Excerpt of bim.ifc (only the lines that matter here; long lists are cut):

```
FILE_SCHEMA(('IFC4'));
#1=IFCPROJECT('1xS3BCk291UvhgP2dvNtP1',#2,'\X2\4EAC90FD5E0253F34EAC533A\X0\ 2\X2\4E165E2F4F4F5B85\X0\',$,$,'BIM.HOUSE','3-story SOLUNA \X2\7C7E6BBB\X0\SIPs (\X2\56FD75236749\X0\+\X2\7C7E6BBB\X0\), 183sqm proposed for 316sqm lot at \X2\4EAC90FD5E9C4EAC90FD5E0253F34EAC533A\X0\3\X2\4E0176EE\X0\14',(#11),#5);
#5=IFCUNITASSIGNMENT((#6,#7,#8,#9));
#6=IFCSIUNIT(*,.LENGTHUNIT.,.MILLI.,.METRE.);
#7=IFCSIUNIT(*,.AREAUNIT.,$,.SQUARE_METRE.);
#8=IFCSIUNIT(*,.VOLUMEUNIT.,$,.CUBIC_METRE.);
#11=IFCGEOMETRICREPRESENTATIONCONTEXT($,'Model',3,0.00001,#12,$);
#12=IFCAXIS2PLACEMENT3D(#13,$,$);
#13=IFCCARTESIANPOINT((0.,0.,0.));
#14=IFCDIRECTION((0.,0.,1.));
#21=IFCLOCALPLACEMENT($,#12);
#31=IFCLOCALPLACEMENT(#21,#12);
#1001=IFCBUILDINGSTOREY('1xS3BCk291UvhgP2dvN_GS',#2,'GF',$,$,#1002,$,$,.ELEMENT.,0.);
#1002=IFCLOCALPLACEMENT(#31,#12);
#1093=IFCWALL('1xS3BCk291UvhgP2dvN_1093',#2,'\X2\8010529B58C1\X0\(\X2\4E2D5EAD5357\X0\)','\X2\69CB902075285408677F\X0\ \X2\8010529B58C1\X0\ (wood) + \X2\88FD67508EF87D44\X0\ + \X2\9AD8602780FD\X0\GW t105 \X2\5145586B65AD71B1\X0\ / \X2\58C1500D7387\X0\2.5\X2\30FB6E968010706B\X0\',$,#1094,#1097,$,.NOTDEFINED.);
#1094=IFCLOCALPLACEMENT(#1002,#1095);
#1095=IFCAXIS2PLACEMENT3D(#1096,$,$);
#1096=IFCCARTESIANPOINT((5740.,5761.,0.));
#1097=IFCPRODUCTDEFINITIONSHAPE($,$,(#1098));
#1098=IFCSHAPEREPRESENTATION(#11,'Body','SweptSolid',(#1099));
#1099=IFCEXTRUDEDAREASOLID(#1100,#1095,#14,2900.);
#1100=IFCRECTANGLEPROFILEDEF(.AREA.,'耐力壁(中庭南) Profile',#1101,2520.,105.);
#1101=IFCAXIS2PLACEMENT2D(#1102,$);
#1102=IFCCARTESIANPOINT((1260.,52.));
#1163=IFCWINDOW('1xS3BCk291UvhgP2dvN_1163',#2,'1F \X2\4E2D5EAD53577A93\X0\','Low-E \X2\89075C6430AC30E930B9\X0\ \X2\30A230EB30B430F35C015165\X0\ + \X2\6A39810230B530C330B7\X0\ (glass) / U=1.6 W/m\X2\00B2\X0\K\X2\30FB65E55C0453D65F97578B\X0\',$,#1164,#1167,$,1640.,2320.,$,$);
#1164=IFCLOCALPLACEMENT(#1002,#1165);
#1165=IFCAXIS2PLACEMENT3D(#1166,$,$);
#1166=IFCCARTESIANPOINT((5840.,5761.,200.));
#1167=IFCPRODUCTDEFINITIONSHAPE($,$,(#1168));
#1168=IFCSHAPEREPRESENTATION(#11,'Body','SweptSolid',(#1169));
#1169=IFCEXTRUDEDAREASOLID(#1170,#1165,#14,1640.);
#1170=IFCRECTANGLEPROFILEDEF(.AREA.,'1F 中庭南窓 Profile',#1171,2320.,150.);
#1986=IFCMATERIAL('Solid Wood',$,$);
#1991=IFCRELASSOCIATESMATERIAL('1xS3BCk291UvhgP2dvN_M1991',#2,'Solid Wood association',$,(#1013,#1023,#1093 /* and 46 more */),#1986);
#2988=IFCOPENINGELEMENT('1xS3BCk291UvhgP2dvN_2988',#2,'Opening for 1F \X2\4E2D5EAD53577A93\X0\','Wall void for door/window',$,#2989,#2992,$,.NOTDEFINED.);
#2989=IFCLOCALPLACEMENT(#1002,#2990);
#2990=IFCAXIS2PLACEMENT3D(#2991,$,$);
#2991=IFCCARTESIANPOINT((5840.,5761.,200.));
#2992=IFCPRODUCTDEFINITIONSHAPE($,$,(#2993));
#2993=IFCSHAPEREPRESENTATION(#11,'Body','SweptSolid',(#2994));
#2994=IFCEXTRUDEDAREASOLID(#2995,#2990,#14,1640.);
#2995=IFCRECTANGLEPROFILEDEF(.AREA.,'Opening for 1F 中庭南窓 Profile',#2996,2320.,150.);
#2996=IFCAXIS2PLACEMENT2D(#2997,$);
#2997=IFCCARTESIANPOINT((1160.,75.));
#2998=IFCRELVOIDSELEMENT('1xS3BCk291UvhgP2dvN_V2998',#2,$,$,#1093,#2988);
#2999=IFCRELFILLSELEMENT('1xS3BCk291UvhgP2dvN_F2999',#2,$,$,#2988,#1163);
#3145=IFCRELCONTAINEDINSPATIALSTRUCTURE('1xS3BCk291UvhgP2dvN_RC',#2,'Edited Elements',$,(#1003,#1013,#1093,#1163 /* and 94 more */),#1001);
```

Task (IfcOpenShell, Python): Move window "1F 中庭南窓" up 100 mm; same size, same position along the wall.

```python
import numpy as np
import ifcopenshell
import ifcopenshell.api.geometry
import ifcopenshell.util.placement
import ifcopenshell.util.unit

model = ifcopenshell.open("bim.ifc")
unit_scale = ifcopenshell.util.unit.calculate_unit_scale(model)

window = model.by_guid("1xS3BCk291UvhgP2dvN_1163")
opening = window.FillsVoids[0].RelatingOpeningElement
dz = 0.1 / unit_scale

shift = np.array([0.0, 0.0, dz])
# The window is not placed relative to its opening, so move both.
for product in (opening, window):
    matrix = ifcopenshell.util.placement.get_local_placement(product.ObjectPlacement)
    matrix[:3, 3] += shift
    ifcopenshell.api.geometry.edit_object_placement(model, product=product, matrix=matrix, is_si=False)

print(f"moved by {dz * unit_scale:+.3f} m")

model.write("bim_v2.ifc")
```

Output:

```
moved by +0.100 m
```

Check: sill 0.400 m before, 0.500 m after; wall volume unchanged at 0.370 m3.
